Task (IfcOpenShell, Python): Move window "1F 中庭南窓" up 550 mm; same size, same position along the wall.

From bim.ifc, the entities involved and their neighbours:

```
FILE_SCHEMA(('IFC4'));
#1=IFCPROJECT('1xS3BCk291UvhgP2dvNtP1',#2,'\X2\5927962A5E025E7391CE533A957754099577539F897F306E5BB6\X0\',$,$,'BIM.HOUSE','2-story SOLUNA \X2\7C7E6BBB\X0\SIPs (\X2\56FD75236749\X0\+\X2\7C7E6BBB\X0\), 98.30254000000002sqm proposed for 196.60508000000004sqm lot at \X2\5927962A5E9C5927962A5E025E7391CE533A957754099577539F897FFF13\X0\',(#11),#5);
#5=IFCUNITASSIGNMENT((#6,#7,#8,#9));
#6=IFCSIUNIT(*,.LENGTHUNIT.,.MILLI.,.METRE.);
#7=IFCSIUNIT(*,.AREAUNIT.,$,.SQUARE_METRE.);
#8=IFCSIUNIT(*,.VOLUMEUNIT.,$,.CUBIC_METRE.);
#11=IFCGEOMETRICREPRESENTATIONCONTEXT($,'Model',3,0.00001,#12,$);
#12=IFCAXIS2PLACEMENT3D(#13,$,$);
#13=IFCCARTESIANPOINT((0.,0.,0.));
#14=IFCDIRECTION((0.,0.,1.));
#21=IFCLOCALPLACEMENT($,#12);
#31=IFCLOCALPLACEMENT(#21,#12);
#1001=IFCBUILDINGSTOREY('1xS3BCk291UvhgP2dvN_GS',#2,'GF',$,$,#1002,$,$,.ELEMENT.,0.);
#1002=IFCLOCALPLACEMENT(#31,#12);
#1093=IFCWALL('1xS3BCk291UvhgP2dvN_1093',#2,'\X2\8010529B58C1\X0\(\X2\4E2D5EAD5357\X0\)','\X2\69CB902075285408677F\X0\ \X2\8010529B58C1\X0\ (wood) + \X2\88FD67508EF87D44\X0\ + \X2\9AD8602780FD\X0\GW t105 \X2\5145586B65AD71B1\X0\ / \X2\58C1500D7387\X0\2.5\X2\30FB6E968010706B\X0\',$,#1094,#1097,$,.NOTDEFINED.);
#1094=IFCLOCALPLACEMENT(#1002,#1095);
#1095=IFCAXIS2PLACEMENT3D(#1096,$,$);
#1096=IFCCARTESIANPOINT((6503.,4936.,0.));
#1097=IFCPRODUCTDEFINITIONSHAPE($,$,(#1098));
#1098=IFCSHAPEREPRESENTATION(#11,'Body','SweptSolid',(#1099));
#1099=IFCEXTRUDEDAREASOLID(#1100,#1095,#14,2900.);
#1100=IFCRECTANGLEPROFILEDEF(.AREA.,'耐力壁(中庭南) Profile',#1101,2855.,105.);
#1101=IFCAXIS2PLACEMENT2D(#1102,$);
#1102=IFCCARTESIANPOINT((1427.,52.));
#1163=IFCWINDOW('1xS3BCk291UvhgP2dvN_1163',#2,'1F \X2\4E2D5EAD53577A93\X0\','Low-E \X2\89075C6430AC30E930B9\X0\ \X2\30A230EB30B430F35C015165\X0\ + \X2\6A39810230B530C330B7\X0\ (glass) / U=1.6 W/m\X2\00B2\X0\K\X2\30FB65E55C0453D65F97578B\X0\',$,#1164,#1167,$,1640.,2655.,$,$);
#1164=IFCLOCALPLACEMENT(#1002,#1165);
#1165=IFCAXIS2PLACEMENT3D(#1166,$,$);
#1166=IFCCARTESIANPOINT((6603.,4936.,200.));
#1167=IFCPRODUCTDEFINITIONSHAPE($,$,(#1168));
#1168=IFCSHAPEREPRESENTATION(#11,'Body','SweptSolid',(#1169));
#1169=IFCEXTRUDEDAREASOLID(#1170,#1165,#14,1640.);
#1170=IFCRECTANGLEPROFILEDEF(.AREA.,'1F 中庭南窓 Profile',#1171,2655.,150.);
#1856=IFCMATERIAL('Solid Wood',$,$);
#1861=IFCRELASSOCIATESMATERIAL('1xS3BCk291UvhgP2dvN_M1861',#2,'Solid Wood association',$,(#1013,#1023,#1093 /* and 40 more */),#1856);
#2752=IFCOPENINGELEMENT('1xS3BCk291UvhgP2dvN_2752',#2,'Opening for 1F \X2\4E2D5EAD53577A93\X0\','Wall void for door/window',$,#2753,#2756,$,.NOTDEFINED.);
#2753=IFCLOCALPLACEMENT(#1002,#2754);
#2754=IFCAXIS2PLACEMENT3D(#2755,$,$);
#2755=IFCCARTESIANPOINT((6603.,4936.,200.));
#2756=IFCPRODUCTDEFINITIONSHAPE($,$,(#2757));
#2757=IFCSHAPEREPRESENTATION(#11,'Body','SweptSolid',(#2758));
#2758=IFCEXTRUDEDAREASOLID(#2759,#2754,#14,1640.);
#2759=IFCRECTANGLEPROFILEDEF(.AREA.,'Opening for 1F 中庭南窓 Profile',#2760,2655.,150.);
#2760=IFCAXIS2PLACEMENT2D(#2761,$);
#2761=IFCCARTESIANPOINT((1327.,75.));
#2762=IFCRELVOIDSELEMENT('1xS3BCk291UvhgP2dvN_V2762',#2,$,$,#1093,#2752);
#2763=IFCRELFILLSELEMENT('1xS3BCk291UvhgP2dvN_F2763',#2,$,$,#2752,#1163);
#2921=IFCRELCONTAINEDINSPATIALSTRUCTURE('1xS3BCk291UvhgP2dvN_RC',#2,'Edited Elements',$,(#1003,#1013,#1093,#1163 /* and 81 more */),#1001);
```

```python
import numpy as np
import ifcopenshell
import ifcopenshell.api.geometry
import ifcopenshell.util.placement
import ifcopenshell.util.unit

model = ifcopenshell.open("bim.ifc")
unit_scale = ifcopenshell.util.unit.calculate_unit_scale(model)

window = model.by_id(1163)
opening = window.FillsVoids[0].RelatingOpeningElement
dz = 550.0

shift = np.array([0.0, 0.0, dz])
# The window is not placed relative to its opening, so move both.
for product in (opening, window):
    matrix = ifcopenshell.util.placement.get_local_placement(product.ObjectPlacement)
    matrix[:3, 3] += shift
    ifcopenshell.api.geometry.edit_object_placement(model, product=product, matrix=matrix, is_si=False)

print(f"moved by {dz * unit_scale:+.3f} m")

model.write("bim_updated.ifc")
```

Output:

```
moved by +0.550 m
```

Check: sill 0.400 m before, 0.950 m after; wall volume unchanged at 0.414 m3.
